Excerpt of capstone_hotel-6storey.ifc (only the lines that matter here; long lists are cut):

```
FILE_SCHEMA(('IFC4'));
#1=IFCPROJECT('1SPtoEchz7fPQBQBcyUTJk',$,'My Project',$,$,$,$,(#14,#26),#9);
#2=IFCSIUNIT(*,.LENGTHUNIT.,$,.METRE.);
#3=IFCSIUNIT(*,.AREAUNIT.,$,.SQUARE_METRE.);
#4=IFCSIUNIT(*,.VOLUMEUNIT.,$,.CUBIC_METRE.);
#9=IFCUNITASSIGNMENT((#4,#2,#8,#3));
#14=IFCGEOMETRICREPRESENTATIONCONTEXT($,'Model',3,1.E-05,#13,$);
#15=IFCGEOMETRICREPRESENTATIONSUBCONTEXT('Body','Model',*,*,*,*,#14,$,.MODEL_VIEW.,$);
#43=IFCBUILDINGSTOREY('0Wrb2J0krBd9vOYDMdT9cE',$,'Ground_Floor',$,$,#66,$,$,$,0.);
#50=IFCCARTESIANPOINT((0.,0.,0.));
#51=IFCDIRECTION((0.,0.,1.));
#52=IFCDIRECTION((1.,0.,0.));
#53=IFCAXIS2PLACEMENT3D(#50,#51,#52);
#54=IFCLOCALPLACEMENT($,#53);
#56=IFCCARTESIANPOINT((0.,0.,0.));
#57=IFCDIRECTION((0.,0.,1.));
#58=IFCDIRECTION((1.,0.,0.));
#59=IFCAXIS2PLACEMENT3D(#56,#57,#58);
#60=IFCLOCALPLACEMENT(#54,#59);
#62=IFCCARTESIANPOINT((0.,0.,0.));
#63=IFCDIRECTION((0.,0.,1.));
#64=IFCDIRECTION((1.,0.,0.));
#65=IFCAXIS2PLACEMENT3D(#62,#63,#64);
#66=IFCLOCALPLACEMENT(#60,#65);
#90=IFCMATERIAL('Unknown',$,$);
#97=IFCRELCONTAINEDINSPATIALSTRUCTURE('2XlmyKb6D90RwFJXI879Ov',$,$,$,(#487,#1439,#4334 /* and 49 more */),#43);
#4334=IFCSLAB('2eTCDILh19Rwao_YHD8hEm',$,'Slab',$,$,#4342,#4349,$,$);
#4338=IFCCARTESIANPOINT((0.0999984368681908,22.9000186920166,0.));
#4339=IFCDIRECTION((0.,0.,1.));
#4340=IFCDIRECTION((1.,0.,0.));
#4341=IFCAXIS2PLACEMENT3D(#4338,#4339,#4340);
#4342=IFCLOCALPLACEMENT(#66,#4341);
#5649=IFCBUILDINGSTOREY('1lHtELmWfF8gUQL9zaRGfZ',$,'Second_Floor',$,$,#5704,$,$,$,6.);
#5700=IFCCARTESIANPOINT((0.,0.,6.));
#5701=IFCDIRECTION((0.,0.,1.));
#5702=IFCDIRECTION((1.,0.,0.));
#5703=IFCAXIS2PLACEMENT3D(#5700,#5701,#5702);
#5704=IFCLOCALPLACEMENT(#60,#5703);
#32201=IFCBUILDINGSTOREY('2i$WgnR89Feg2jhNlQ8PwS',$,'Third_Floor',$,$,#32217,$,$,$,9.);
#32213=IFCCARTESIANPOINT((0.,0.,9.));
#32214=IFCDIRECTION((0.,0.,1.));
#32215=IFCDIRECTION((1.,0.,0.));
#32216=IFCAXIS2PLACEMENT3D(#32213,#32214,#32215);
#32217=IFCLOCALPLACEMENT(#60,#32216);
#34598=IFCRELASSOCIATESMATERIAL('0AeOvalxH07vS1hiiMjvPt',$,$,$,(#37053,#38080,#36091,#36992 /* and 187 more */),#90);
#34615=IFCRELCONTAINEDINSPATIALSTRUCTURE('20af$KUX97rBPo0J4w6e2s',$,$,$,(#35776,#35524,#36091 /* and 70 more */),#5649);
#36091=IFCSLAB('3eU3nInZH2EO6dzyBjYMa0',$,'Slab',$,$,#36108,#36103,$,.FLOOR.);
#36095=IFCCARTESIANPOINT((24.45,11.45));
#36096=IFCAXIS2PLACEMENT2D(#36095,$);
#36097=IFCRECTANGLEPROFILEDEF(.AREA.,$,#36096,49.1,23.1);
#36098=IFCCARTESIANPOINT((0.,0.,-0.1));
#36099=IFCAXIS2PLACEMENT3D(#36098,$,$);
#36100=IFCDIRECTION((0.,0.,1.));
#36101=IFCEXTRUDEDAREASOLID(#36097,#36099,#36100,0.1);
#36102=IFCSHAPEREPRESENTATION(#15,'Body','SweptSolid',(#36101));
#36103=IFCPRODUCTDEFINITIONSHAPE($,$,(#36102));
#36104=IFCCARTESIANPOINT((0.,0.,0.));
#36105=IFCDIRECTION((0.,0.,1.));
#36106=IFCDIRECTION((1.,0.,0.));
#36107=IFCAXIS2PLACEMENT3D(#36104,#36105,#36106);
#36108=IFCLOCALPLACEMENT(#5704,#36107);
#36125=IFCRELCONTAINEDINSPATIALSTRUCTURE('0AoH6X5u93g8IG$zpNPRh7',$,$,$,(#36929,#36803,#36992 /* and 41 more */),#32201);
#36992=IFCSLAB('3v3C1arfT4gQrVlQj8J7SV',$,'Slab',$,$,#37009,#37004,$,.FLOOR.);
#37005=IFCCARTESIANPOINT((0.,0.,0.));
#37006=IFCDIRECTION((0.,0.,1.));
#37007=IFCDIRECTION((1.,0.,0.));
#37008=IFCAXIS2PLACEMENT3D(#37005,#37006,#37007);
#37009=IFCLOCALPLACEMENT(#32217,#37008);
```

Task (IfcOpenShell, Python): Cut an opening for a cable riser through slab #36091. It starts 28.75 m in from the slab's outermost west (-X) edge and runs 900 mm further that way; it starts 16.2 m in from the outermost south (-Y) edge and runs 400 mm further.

```python
import numpy as np
import ifcopenshell
import ifcopenshell.api.feature
import ifcopenshell.api.geometry
import ifcopenshell.api.root
import ifcopenshell.geom
import ifcopenshell.util.placement
import ifcopenshell.util.representation
import ifcopenshell.util.shape
import ifcopenshell.util.unit

model = ifcopenshell.open("capstone_hotel-6storey.ifc")
unit_scale = ifcopenshell.util.unit.calculate_unit_scale(model)
settings = ifcopenshell.geom.settings()


def volume(element):
    """Net volume in cubic metres, openings subtracted."""
    shape = ifcopenshell.geom.create_shape(settings, element)
    return ifcopenshell.util.shape.get_volume(shape.geometry)


slab = model.by_guid("3eU3nInZH2EO6dzyBjYMa0")
before = volume(slab)

# Extent in the slab's own axes, in metres. The edges named are its -X and -Y sides.
slab_shape = ifcopenshell.geom.create_shape(settings, slab)
vertices = ifcopenshell.util.shape.get_vertices(slab_shape.geometry)
x_min, y_min, bottom = vertices.min(axis=0)
top = vertices[:, 2].max()

opening = ifcopenshell.api.root.create_entity(model, ifc_class="IfcOpeningElement", name="Cable riser opening", predefined_type="OPENING")
context = ifcopenshell.util.representation.get_context(model, "Model", "Body", "MODEL_VIEW")
width, depth = 0.9, 0.4
outline = [(0.0, 0.0), (width, 0.0), (width, depth), (0.0, depth), (0.0, 0.0)]
# Overshoot both faces by 50 mm so the cut is clean.
shape = ifcopenshell.api.geometry.add_slab_representation(
    model, context=context, depth=top - bottom + 0.1, polyline=outline
)
ifcopenshell.api.geometry.assign_representation(model, product=opening, representation=shape)

matrix = ifcopenshell.util.placement.get_local_placement(slab.ObjectPlacement)
matrix[:, 3] = matrix @ np.append(np.array([x_min + 28.75, y_min + 16.2, bottom - 0.05]) / unit_scale, 1.0)
ifcopenshell.api.geometry.edit_object_placement(model, product=opening, matrix=matrix, is_si=False)
ifcopenshell.api.feature.add_feature(model, feature=opening, element=slab)

after = volume(slab)

print(f"slab volume {before:.3f} -> {after:.3f} m3")

model.write("capstone_hotel-6storey_rev.ifc")
```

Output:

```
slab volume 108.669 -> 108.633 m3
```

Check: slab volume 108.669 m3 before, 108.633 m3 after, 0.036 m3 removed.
